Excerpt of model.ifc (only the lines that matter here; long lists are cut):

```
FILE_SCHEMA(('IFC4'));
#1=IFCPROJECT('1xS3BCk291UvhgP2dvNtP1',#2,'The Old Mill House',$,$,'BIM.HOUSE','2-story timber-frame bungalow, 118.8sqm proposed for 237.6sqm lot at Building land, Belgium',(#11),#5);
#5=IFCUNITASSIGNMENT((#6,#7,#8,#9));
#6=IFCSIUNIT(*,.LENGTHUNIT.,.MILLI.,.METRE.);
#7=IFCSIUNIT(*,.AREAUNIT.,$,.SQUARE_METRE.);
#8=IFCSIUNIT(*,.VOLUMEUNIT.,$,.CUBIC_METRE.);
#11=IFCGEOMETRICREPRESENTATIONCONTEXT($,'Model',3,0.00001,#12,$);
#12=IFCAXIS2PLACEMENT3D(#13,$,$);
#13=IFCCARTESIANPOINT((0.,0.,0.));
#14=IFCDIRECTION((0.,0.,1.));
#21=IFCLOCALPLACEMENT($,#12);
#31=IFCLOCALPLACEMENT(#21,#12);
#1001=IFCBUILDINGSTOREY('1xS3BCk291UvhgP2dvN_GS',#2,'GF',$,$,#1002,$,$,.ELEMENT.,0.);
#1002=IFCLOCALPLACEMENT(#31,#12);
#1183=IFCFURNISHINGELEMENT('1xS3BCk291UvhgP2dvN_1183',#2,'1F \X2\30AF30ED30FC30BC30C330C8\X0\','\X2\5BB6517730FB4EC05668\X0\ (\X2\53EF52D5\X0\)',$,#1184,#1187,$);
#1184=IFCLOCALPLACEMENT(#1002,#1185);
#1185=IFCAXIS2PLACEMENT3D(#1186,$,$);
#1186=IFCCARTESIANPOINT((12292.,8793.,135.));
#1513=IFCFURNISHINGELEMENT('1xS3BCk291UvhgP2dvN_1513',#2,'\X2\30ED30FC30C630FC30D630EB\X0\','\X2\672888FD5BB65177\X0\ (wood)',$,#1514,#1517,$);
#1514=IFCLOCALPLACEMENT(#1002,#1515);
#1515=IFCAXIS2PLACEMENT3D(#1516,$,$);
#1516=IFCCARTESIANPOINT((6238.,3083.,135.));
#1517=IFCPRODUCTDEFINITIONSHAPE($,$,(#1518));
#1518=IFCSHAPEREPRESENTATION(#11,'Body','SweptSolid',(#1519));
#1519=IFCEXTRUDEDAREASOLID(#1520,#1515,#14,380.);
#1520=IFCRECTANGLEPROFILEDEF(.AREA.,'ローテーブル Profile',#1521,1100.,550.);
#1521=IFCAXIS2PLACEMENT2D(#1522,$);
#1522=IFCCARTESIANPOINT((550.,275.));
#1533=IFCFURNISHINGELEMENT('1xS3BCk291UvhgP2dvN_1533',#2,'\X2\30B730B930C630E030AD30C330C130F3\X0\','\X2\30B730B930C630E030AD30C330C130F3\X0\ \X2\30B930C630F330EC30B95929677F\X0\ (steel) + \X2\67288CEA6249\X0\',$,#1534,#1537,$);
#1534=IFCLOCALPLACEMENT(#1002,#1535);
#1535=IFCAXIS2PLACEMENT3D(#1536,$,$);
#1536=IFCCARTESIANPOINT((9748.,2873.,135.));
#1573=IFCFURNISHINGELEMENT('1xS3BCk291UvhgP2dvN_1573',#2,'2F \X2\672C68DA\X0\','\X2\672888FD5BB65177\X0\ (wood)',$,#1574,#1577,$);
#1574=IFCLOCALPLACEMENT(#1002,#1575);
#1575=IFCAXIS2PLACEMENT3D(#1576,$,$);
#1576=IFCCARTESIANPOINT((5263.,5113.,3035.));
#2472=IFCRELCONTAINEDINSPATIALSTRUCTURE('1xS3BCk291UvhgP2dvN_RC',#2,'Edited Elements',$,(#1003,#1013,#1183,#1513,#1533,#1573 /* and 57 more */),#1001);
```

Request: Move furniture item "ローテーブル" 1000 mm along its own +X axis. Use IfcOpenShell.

```python
import ifcopenshell
import ifcopenshell.api.geometry
import ifcopenshell.util.placement
import ifcopenshell.util.unit

model = ifcopenshell.open("model.ifc")
unit_scale = ifcopenshell.util.unit.calculate_unit_scale(model)

item = model.by_guid("1xS3BCk291UvhgP2dvN_1513")
matrix = ifcopenshell.util.placement.get_local_placement(item.ObjectPlacement)
matrix[:3, 3] += matrix[:3, 0] * 1 / unit_scale
ifcopenshell.api.geometry.edit_object_placement(model, product=item, matrix=matrix, is_si=False)

print(ifcopenshell.util.placement.get_local_placement(item.ObjectPlacement).round(3) + 0.0)

model.write("model_v2.ifc")
```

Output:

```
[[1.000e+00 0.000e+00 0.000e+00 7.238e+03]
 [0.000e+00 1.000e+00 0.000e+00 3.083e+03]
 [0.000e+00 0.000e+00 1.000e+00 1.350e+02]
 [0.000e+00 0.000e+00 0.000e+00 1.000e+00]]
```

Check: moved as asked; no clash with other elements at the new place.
